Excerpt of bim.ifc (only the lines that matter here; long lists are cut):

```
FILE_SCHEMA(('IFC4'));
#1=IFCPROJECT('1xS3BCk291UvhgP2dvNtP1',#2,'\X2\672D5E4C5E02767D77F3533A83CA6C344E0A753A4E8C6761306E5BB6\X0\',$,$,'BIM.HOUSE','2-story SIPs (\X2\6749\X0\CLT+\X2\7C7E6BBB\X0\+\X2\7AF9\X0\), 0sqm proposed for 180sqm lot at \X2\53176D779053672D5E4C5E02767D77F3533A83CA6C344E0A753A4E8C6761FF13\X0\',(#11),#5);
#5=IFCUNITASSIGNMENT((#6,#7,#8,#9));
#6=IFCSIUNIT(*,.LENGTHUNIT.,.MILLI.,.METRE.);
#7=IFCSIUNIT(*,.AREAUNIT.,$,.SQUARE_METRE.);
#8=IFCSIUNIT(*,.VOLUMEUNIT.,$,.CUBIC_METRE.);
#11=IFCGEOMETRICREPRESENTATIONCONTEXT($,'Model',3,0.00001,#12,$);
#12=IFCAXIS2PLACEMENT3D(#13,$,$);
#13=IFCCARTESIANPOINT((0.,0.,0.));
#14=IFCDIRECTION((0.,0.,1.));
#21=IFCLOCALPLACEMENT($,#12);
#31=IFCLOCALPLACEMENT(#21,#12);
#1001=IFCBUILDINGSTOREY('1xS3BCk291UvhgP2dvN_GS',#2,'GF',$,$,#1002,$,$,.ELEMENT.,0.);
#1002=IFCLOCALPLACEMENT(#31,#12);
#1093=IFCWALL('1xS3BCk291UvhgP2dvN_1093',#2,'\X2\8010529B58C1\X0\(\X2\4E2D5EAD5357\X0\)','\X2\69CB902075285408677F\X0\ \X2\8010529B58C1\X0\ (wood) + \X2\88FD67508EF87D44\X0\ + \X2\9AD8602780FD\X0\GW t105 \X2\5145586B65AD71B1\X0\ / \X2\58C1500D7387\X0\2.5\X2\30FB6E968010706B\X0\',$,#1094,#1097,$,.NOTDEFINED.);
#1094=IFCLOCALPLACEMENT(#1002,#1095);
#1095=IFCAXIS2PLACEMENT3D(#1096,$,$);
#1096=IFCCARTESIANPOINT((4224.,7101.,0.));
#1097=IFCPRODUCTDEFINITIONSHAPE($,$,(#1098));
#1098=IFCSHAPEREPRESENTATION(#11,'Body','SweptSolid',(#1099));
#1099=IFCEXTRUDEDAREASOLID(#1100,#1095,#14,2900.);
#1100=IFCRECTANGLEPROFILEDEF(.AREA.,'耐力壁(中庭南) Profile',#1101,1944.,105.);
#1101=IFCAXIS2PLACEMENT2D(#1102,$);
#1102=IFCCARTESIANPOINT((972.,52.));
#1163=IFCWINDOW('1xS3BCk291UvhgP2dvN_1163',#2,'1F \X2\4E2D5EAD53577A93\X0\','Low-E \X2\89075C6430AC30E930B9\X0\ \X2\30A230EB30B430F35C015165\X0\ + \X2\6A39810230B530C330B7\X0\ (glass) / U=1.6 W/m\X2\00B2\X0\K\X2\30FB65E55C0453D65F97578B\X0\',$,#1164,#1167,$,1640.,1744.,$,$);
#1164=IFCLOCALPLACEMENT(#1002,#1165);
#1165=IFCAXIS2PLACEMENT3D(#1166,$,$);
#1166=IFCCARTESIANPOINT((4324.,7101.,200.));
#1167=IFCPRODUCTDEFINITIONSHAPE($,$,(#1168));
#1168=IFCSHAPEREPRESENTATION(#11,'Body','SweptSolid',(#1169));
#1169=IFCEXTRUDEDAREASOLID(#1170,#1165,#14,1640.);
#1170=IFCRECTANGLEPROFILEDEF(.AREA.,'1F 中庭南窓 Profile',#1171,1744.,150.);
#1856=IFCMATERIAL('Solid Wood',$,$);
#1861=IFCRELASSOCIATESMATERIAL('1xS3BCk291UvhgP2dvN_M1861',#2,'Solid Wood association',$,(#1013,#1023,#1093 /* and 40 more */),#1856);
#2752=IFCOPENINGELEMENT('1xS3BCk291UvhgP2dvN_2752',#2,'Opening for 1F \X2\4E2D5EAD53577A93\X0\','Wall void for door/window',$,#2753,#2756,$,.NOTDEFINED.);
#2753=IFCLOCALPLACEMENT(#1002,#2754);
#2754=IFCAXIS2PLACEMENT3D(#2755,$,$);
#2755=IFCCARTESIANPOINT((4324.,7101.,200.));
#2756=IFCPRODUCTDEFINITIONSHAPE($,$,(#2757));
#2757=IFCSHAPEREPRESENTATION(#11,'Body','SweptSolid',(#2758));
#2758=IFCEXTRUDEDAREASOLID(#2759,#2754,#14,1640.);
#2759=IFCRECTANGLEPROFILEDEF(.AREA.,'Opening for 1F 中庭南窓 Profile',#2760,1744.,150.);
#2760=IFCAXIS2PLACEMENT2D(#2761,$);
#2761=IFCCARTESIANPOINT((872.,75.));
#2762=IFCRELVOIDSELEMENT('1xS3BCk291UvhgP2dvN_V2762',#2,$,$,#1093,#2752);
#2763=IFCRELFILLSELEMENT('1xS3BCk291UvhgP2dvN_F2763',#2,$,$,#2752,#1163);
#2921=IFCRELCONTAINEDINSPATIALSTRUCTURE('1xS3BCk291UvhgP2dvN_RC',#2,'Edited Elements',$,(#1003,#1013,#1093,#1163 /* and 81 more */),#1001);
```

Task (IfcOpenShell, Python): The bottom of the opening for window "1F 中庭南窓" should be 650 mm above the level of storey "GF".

```python
import numpy as np
import ifcopenshell
import ifcopenshell.api.geometry
import ifcopenshell.geom
import ifcopenshell.util.element
import ifcopenshell.util.placement
import ifcopenshell.util.shape
import ifcopenshell.util.unit

model = ifcopenshell.open("bim.ifc")
unit_scale = ifcopenshell.util.unit.calculate_unit_scale(model)

window = model.by_id(1163)
opening = window.FillsVoids[0].RelatingOpeningElement
storey = ifcopenshell.util.element.get_container(window, ifc_class="IfcBuildingStorey")
level = ifcopenshell.util.placement.get_local_placement(storey.ObjectPlacement)[2, 3]

# The opening's origin need not be at the sill, so measure its lowest point.
shape = ifcopenshell.geom.create_shape(ifcopenshell.geom.settings(), opening)
bottom = ifcopenshell.util.shape.get_shape_bottom_elevation(shape, shape.geometry) / unit_scale
dz = level + 0.65 / unit_scale - bottom

shift = np.array([0.0, 0.0, dz])
# The window is not placed relative to its opening, so move both.
for product in (opening, window):
    matrix = ifcopenshell.util.placement.get_local_placement(product.ObjectPlacement)
    matrix[:3, 3] += shift
    ifcopenshell.api.geometry.edit_object_placement(model, product=product, matrix=matrix, is_si=False)

print(f"moved by {dz * unit_scale:+.3f} m")

model.write("bim_v2.ifc")
```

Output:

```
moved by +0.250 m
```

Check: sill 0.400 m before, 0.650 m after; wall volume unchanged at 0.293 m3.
